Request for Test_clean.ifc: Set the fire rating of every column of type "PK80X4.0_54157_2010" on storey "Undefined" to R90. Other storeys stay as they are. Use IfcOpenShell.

First a look at what the model holds.

```python
import ifcopenshell
import ifcopenshell.util.element

model = ifcopenshell.open("Test_clean.ifc")
print(model.schema)
storey = next(s for s in model.by_type("IfcBuildingStorey") if s.Name == "Undefined")
columns = [e for e in ifcopenshell.util.element.get_decomposition(storey) if e.is_a("IfcColumn")]
seen = {}
for e in columns:
    element_type = ifcopenshell.util.element.get_type(e)
    key = (element_type.Name if element_type != e and element_type else None, ifcopenshell.util.element.get_pset(e, "Pset_ColumnCommon", "FireRating"))
    seen[key] = seen.get(key, 0) + 1
for (name, value), count in sorted(seen.items(), key=str):
    print(count, "x", name, "|", value)
```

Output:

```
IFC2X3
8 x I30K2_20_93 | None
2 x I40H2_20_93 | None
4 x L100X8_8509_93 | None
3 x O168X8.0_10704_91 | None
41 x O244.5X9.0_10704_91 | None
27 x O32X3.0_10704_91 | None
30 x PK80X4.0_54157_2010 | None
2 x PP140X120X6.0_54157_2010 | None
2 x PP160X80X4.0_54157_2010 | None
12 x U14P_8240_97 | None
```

```python
import ifcopenshell
import ifcopenshell.api.pset
import ifcopenshell.util.element

model = ifcopenshell.open("Test_clean.ifc")

storey = next(s for s in model.by_type("IfcBuildingStorey") if s.Name == "Undefined")
columns = [e for e in ifcopenshell.util.element.get_decomposition(storey) if e.is_a("IfcColumn")]

count = 0
for e in columns:
    element_type = ifcopenshell.util.element.get_type(e)
    if element_type in (None, e) or element_type.Name != "PK80X4.0_54157_2010":
        continue
    found = ifcopenshell.util.element.get_pset(e, "Pset_ColumnCommon", should_inherit=False)
    if found:
        pset = model.by_id(found["id"])
        if len(ifcopenshell.util.element.get_elements_by_pset(pset)) > 1:
            pset = ifcopenshell.api.pset.unshare_pset(model, products=[e], pset=pset)[0]
    else:
        pset = ifcopenshell.api.pset.add_pset(model, product=e, name="Pset_ColumnCommon")
    ifcopenshell.api.pset.edit_pset(model, pset=pset, properties={"FireRating": "R90"})
    count += 1

print(count, "columns updated")

model.write("Test_clean_edited.ifc")
```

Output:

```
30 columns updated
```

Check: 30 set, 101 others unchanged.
